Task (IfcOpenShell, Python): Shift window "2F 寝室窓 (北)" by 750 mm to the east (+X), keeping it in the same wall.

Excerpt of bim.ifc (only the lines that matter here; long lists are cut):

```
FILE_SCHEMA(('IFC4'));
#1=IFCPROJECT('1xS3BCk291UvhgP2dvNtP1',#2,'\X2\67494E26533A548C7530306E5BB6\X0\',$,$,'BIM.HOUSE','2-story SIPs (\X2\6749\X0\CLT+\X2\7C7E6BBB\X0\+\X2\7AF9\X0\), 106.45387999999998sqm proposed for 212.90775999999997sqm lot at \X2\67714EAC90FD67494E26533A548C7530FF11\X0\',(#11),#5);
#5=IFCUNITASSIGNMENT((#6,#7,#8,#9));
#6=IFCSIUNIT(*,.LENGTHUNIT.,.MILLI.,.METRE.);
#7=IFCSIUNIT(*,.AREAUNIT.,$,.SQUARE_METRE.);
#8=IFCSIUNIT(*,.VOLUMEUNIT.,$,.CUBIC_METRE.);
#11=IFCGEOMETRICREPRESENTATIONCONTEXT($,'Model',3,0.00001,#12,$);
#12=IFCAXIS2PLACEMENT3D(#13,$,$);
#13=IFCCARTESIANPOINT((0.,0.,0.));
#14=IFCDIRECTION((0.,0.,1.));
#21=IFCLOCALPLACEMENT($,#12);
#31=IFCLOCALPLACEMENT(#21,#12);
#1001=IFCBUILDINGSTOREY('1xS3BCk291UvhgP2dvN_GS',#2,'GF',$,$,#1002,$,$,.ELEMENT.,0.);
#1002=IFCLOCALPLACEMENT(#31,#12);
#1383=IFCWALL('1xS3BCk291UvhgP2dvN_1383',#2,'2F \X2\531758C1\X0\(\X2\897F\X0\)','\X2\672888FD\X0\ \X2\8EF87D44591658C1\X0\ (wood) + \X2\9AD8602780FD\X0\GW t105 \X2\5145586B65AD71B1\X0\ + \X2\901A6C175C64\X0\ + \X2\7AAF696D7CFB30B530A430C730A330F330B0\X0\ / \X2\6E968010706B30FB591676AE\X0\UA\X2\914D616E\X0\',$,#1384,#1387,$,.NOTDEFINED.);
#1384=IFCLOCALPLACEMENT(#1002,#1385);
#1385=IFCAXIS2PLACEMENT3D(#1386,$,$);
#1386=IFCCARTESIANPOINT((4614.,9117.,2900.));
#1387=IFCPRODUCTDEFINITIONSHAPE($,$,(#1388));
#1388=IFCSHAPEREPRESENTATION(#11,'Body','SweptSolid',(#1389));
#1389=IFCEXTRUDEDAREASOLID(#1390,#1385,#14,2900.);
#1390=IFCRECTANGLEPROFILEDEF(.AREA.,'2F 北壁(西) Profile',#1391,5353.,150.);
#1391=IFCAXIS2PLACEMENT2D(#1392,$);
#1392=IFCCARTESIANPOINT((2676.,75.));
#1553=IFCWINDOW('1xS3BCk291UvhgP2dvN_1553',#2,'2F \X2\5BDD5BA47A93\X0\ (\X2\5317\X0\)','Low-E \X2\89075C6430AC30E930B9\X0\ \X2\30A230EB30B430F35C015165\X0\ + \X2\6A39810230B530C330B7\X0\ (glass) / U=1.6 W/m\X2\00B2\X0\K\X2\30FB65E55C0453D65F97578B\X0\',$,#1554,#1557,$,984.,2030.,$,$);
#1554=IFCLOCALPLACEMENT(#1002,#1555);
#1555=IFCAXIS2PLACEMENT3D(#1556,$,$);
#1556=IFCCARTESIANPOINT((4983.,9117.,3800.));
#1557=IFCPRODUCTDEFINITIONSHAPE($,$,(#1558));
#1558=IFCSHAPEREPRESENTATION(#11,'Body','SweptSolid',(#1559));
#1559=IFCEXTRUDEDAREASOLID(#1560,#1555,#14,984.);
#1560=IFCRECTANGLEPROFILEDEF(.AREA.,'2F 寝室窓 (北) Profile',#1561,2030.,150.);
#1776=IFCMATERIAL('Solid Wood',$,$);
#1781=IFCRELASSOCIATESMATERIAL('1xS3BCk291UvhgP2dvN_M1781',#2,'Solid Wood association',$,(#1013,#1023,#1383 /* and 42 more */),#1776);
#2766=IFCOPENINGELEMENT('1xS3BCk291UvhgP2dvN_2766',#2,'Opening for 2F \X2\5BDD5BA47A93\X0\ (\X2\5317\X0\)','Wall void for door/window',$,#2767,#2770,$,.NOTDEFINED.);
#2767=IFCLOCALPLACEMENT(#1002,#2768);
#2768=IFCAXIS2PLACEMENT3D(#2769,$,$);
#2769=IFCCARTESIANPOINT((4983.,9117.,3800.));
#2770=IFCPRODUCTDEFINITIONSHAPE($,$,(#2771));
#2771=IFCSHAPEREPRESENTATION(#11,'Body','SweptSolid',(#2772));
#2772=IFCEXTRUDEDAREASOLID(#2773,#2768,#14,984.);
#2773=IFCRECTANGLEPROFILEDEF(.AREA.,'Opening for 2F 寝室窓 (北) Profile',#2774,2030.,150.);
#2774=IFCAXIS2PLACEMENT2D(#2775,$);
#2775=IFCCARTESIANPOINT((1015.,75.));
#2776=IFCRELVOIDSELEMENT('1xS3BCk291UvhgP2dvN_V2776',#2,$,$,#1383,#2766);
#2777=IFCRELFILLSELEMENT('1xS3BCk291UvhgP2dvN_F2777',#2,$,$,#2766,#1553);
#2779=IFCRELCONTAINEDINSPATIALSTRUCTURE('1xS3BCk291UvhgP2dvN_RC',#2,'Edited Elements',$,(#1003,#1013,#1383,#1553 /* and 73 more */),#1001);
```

```python
import ifcopenshell
import ifcopenshell.api.geometry
import ifcopenshell.util.placement
import ifcopenshell.util.unit

model = ifcopenshell.open("bim.ifc")
unit_scale = ifcopenshell.util.unit.calculate_unit_scale(model)

window = model.by_guid("1xS3BCk291UvhgP2dvN_1553")
opening = window.FillsVoids[0].RelatingOpeningElement
wall = opening.VoidsElements[0].RelatingBuildingElement

wall_matrix = ifcopenshell.util.placement.get_local_placement(wall.ObjectPlacement)
shift = wall_matrix[:3, 0] * 0.75 / unit_scale
before = ifcopenshell.util.placement.get_local_placement(window.ObjectPlacement)[:3, 3].copy()

# The window is not placed relative to its opening, so move both.
for product in (opening, window):
    matrix = ifcopenshell.util.placement.get_local_placement(product.ObjectPlacement)
    matrix[:3, 3] += shift
    ifcopenshell.api.geometry.edit_object_placement(model, product=product, matrix=matrix, is_si=False)

after = ifcopenshell.util.placement.get_local_placement(window.ObjectPlacement)[:3, 3]
print("window moved by", (after - before).round(3) + 0.0)

model.write("bim_edited.ifc")
```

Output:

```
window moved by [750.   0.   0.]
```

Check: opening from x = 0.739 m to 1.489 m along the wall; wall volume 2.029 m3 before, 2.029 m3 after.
